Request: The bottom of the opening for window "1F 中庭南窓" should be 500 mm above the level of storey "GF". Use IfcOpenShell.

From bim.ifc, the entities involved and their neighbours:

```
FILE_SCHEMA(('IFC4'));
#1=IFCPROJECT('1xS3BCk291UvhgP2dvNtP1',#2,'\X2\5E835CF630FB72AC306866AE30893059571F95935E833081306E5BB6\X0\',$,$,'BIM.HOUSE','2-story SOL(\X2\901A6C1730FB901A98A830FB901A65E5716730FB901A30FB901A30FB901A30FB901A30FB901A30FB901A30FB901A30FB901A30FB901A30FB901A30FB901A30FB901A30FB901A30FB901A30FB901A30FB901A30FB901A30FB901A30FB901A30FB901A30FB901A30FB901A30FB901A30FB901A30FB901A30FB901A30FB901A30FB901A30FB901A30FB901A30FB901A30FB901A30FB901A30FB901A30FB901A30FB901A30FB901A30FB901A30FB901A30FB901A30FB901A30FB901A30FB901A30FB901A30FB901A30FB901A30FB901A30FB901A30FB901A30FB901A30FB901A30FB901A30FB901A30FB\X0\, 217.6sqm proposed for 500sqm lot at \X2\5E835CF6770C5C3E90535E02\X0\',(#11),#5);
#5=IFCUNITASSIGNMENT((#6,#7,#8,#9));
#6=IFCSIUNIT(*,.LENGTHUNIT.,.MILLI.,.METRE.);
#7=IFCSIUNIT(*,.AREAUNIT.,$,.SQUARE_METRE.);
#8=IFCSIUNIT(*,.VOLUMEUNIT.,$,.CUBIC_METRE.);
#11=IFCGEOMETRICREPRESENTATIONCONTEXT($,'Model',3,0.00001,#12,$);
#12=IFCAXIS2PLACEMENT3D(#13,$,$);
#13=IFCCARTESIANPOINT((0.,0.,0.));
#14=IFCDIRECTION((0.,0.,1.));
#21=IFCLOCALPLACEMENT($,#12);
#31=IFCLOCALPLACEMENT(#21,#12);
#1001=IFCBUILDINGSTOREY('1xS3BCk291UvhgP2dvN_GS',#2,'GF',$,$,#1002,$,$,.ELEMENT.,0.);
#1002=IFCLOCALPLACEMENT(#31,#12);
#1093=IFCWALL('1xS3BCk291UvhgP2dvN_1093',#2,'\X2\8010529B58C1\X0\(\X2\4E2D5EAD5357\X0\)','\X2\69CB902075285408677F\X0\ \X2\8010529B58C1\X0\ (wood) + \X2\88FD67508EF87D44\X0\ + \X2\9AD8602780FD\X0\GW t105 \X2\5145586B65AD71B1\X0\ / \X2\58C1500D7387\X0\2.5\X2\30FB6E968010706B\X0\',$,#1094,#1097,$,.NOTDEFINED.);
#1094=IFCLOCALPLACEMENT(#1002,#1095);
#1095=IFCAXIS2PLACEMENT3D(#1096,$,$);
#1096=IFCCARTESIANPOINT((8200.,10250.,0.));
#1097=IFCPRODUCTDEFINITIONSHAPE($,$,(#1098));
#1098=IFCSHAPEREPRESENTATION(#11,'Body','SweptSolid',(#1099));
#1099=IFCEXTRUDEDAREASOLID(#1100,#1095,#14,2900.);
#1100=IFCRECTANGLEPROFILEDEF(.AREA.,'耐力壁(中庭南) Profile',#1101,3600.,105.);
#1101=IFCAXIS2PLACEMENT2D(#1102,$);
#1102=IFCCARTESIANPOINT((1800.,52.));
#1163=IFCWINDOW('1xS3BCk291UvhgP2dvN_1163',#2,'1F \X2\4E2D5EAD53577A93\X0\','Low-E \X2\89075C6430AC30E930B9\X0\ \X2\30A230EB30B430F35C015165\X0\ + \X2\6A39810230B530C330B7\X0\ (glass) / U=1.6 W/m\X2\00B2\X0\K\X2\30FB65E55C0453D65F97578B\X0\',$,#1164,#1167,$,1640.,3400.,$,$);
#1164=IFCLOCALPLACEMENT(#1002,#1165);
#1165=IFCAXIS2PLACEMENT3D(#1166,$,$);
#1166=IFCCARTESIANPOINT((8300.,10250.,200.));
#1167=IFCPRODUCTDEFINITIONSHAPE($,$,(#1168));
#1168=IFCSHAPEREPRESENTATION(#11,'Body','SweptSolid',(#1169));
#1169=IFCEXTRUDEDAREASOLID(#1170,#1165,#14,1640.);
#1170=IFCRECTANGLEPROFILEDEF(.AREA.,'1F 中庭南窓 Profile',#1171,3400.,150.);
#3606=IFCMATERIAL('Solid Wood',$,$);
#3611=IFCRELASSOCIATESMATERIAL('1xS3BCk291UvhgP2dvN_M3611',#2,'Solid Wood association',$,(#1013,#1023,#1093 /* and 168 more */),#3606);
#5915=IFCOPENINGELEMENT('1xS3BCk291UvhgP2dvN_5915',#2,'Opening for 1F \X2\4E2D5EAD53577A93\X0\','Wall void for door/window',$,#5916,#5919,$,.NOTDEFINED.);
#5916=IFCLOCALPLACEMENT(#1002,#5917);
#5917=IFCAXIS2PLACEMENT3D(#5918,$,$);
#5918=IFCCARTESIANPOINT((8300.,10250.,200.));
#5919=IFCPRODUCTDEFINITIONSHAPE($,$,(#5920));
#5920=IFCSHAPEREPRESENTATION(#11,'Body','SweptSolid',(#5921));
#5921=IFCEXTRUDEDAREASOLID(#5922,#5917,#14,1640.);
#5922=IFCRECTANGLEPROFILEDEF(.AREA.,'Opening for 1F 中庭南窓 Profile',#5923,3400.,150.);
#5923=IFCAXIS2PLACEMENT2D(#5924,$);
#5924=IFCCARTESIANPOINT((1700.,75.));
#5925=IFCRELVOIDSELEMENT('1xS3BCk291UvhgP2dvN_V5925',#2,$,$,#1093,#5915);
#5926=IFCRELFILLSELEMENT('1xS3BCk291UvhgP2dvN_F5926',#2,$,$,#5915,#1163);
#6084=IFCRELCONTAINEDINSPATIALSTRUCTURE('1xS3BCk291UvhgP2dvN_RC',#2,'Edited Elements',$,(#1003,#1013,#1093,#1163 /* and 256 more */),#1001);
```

```python
import numpy as np
import ifcopenshell
import ifcopenshell.api.geometry
import ifcopenshell.geom
import ifcopenshell.util.element
import ifcopenshell.util.placement
import ifcopenshell.util.shape
import ifcopenshell.util.unit

model = ifcopenshell.open("bim.ifc")
unit_scale = ifcopenshell.util.unit.calculate_unit_scale(model)

window = model.by_guid("1xS3BCk291UvhgP2dvN_1163")
opening = window.FillsVoids[0].RelatingOpeningElement
storey = ifcopenshell.util.element.get_container(window, ifc_class="IfcBuildingStorey")
level = ifcopenshell.util.placement.get_local_placement(storey.ObjectPlacement)[2, 3]

# The opening's origin need not be at the sill, so measure its lowest point.
shape = ifcopenshell.geom.create_shape(ifcopenshell.geom.settings(), opening)
bottom = ifcopenshell.util.shape.get_shape_bottom_elevation(shape, shape.geometry) / unit_scale
dz = level + 0.5 / unit_scale - bottom

shift = np.array([0.0, 0.0, dz])
# The window is not placed relative to its opening, so move both.
for product in (opening, window):
    matrix = ifcopenshell.util.placement.get_local_placement(product.ObjectPlacement)
    matrix[:3, 3] += shift
    ifcopenshell.api.geometry.edit_object_placement(model, product=product, matrix=matrix, is_si=False)

print(f"moved by {dz * unit_scale:+.3f} m")

model.write("bim_updated.ifc")
```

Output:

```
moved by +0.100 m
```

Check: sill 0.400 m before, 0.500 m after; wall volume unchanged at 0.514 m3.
